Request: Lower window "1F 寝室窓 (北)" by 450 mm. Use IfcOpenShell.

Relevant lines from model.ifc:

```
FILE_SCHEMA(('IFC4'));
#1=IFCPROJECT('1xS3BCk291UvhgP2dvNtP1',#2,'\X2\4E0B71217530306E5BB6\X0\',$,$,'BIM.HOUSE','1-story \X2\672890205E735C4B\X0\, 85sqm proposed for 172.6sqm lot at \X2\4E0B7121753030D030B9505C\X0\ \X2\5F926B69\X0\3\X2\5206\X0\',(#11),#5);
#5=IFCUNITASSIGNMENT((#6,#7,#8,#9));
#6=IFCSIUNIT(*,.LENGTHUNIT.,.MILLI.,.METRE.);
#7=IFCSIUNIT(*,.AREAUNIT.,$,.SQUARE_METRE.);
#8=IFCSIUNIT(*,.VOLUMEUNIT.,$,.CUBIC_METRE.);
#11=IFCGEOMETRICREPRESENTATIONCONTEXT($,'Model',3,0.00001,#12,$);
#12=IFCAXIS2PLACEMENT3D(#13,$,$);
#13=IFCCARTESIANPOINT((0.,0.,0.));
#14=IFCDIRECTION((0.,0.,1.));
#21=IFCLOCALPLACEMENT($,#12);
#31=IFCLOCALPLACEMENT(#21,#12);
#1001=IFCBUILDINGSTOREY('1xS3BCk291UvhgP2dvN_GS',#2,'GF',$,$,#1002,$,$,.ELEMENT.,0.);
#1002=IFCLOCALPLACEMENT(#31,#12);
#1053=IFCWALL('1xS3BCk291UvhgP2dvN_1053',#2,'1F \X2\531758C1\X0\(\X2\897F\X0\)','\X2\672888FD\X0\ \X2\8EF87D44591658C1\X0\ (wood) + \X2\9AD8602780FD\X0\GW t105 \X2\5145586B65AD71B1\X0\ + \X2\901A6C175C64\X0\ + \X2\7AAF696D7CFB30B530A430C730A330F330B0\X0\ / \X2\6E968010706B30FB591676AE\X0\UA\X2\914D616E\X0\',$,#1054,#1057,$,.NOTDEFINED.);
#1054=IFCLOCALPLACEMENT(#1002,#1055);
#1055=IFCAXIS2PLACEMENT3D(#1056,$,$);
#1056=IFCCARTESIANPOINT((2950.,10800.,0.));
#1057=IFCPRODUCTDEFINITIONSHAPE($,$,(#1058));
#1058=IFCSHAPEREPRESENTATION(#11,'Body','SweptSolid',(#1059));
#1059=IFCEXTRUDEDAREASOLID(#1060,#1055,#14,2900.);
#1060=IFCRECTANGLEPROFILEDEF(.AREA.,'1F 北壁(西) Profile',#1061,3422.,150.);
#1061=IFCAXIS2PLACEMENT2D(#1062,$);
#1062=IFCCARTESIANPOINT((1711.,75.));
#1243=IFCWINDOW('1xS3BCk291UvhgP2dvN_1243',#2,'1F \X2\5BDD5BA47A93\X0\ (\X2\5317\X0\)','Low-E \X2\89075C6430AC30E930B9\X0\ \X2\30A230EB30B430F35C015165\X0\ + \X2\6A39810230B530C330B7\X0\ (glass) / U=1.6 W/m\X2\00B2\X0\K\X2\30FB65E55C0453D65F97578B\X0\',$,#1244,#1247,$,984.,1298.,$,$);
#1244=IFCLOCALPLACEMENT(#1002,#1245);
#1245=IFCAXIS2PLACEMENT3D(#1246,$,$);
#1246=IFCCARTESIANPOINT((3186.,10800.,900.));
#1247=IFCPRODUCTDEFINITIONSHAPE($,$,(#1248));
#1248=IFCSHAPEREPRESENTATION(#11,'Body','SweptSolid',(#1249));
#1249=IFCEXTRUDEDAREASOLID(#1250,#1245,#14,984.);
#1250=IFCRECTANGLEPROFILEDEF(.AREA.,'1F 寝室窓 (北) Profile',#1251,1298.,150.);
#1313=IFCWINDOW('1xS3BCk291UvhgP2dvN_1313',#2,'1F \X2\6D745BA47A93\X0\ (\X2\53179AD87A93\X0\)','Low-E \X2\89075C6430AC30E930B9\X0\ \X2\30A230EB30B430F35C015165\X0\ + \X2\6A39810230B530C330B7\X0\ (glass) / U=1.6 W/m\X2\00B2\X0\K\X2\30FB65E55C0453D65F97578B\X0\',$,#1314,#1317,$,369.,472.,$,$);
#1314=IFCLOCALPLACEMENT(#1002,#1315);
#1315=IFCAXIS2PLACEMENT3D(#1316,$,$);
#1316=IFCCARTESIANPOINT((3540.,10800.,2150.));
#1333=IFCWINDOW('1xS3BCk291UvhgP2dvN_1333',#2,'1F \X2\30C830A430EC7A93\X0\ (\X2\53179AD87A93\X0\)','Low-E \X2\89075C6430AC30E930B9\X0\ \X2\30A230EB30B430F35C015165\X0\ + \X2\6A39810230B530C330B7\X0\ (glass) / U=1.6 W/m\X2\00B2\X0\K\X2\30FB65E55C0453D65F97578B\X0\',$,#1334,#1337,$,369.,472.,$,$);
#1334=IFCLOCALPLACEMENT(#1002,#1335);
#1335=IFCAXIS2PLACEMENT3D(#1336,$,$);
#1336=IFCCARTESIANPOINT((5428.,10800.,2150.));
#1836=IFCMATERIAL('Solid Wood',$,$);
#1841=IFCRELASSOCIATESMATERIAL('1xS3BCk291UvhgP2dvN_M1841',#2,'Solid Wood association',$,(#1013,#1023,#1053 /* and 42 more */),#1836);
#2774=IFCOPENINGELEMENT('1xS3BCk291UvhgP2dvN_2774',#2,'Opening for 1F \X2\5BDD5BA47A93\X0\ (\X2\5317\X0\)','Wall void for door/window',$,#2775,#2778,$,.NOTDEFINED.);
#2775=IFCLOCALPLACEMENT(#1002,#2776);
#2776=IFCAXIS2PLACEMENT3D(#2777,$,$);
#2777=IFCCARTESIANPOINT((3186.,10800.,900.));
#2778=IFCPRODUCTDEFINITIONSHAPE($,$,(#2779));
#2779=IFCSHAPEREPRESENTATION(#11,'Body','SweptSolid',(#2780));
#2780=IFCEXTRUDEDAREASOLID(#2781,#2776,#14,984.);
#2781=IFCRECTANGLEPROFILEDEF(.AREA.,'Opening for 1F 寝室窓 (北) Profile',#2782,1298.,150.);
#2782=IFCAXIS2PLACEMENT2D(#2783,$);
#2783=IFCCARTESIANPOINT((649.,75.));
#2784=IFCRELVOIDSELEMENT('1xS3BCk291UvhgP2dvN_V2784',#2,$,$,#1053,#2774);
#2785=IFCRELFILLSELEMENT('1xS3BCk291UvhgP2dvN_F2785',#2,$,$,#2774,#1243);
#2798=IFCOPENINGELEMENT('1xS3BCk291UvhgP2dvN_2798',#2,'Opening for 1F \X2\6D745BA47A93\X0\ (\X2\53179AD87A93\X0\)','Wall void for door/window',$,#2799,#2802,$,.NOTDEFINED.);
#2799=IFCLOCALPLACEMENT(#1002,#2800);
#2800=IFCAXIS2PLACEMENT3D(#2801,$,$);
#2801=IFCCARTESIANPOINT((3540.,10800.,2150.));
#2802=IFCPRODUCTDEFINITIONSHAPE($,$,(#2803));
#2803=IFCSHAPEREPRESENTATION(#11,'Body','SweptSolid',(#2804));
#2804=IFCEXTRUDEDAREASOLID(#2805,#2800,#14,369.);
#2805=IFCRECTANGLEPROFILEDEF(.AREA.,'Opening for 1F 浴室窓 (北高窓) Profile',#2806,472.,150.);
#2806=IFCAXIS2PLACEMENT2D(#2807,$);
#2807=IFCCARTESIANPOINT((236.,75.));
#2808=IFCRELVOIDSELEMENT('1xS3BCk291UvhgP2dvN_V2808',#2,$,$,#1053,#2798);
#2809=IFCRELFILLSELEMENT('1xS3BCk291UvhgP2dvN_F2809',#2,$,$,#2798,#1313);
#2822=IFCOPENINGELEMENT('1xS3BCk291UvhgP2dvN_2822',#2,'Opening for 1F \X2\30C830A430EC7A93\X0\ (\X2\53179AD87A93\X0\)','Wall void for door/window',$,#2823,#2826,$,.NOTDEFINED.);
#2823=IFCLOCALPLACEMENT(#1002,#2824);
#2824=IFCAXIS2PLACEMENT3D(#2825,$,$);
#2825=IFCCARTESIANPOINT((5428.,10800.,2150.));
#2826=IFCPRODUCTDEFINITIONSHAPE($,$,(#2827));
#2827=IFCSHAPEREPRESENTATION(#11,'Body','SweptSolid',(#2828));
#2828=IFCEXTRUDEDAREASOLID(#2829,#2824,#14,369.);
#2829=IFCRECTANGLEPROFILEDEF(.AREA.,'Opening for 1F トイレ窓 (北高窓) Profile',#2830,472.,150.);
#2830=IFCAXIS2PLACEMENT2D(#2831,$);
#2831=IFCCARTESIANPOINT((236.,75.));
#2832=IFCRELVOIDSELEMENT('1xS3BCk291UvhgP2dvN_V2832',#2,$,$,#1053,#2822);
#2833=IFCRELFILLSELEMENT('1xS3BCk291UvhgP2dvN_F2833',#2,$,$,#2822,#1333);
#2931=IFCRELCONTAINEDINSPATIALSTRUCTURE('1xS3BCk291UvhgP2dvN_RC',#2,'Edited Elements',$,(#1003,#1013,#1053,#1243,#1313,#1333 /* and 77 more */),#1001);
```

```python
import numpy as np
import ifcopenshell
import ifcopenshell.api.geometry
import ifcopenshell.util.placement
import ifcopenshell.util.unit

model = ifcopenshell.open("model.ifc")
unit_scale = ifcopenshell.util.unit.calculate_unit_scale(model)

window = model.by_id(1243)
opening = window.FillsVoids[0].RelatingOpeningElement
dz = -450.0

shift = np.array([0.0, 0.0, dz])
# The window is not placed relative to its opening, so move both.
for product in (opening, window):
    matrix = ifcopenshell.util.placement.get_local_placement(product.ObjectPlacement)
    matrix[:3, 3] += shift
    ifcopenshell.api.geometry.edit_object_placement(model, product=product, matrix=matrix, is_si=False)

print(f"moved by {dz * unit_scale:+.3f} m")

model.write("model_v2.ifc")
```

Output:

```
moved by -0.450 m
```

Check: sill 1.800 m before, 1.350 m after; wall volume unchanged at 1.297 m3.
